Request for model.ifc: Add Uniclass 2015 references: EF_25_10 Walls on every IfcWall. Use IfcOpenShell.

First a look at what the model holds.

```python
import ifcopenshell

model = ifcopenshell.open("model.ifc")
print(model.schema)
print("classifications:", [c.Name for c in model.by_type("IfcClassification")])
for ifc_class in ("IfcDoor", "IfcRoof", "IfcStair", "IfcWall", "IfcWindow"):
    print(ifc_class, len(model.by_type(ifc_class)))
```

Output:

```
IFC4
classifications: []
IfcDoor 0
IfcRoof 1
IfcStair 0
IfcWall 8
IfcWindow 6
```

```python
import ifcopenshell
import ifcopenshell.api.classification

model = ifcopenshell.open("model.ifc")

system = ifcopenshell.api.classification.add_classification(model, classification="Uniclass 2015")

codes = {
    "IfcWall": ("EF_25_10", "Walls"),
}
for ifc_class, (code, name) in codes.items():
    products = model.by_type(ifc_class)
    ifcopenshell.api.classification.add_reference(
        model, products=products, classification=system, identification=code, name=name
    )
    print(code, len(products))

model.write("model_v2.ifc")
```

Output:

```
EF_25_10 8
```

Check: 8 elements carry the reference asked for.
